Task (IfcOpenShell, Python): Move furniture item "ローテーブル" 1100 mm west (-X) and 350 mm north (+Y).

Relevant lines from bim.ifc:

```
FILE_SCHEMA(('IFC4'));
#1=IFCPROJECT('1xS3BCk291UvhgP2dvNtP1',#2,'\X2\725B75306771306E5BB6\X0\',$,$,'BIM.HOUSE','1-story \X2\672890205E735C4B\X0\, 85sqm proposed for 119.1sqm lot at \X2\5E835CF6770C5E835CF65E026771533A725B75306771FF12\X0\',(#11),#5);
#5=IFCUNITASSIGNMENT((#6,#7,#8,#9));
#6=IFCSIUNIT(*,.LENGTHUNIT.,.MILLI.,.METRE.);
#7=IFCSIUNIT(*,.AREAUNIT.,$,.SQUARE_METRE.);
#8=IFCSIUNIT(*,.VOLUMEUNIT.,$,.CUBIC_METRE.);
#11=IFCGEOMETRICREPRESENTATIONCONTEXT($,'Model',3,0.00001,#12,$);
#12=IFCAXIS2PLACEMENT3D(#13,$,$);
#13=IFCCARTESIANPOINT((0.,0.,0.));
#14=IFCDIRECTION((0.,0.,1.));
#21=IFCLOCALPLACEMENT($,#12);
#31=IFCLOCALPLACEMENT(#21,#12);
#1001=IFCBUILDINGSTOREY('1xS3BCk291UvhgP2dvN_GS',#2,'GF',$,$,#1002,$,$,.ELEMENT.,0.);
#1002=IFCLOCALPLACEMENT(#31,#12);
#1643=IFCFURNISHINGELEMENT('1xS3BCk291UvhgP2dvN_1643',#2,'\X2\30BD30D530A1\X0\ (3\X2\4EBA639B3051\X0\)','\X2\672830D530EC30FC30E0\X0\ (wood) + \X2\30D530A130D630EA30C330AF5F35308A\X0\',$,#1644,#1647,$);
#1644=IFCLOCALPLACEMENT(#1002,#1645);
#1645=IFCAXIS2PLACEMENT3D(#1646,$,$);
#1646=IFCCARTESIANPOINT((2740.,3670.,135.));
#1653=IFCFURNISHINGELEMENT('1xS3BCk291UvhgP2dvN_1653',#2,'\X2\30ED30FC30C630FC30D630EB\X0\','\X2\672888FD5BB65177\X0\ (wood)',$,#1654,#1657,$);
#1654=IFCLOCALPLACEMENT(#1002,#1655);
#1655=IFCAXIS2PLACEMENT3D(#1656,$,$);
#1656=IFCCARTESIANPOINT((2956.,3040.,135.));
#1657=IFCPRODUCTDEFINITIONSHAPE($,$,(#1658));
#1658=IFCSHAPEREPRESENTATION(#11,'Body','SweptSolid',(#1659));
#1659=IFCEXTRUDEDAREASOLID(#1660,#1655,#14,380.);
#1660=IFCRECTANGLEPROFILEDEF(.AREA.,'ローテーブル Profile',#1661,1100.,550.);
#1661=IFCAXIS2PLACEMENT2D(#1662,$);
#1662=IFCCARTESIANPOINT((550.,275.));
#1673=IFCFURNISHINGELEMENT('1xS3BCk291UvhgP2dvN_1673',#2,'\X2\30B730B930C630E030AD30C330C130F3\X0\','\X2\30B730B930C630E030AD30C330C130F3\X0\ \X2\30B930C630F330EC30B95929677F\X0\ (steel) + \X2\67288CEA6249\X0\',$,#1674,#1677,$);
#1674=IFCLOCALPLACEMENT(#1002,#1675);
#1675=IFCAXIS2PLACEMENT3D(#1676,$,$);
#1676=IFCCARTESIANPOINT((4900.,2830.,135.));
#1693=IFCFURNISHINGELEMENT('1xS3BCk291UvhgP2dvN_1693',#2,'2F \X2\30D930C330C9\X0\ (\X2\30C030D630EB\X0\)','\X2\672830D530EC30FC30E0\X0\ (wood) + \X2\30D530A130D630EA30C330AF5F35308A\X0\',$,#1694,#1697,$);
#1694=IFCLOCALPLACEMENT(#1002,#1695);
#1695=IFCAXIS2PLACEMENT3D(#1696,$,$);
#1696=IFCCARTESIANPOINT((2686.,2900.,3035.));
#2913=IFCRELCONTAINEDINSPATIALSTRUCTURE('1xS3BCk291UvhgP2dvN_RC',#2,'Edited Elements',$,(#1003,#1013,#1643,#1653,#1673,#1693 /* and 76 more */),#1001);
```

```python
import ifcopenshell
import ifcopenshell.api.geometry
import ifcopenshell.util.placement

model = ifcopenshell.open("bim.ifc")

item = model.by_guid("1xS3BCk291UvhgP2dvN_1653")
matrix = ifcopenshell.util.placement.get_local_placement(item.ObjectPlacement)
matrix[0, 3] -= 1100.0
matrix[1, 3] += 350.0
ifcopenshell.api.geometry.edit_object_placement(model, product=item, matrix=matrix, is_si=False)

print(ifcopenshell.util.placement.get_local_placement(item.ObjectPlacement).round(3) + 0.0)

model.write("bim_v2.ifc")
```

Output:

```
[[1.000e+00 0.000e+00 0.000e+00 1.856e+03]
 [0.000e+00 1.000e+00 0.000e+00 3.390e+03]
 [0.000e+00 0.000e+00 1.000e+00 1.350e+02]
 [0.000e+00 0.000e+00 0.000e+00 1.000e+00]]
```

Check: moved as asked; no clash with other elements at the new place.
